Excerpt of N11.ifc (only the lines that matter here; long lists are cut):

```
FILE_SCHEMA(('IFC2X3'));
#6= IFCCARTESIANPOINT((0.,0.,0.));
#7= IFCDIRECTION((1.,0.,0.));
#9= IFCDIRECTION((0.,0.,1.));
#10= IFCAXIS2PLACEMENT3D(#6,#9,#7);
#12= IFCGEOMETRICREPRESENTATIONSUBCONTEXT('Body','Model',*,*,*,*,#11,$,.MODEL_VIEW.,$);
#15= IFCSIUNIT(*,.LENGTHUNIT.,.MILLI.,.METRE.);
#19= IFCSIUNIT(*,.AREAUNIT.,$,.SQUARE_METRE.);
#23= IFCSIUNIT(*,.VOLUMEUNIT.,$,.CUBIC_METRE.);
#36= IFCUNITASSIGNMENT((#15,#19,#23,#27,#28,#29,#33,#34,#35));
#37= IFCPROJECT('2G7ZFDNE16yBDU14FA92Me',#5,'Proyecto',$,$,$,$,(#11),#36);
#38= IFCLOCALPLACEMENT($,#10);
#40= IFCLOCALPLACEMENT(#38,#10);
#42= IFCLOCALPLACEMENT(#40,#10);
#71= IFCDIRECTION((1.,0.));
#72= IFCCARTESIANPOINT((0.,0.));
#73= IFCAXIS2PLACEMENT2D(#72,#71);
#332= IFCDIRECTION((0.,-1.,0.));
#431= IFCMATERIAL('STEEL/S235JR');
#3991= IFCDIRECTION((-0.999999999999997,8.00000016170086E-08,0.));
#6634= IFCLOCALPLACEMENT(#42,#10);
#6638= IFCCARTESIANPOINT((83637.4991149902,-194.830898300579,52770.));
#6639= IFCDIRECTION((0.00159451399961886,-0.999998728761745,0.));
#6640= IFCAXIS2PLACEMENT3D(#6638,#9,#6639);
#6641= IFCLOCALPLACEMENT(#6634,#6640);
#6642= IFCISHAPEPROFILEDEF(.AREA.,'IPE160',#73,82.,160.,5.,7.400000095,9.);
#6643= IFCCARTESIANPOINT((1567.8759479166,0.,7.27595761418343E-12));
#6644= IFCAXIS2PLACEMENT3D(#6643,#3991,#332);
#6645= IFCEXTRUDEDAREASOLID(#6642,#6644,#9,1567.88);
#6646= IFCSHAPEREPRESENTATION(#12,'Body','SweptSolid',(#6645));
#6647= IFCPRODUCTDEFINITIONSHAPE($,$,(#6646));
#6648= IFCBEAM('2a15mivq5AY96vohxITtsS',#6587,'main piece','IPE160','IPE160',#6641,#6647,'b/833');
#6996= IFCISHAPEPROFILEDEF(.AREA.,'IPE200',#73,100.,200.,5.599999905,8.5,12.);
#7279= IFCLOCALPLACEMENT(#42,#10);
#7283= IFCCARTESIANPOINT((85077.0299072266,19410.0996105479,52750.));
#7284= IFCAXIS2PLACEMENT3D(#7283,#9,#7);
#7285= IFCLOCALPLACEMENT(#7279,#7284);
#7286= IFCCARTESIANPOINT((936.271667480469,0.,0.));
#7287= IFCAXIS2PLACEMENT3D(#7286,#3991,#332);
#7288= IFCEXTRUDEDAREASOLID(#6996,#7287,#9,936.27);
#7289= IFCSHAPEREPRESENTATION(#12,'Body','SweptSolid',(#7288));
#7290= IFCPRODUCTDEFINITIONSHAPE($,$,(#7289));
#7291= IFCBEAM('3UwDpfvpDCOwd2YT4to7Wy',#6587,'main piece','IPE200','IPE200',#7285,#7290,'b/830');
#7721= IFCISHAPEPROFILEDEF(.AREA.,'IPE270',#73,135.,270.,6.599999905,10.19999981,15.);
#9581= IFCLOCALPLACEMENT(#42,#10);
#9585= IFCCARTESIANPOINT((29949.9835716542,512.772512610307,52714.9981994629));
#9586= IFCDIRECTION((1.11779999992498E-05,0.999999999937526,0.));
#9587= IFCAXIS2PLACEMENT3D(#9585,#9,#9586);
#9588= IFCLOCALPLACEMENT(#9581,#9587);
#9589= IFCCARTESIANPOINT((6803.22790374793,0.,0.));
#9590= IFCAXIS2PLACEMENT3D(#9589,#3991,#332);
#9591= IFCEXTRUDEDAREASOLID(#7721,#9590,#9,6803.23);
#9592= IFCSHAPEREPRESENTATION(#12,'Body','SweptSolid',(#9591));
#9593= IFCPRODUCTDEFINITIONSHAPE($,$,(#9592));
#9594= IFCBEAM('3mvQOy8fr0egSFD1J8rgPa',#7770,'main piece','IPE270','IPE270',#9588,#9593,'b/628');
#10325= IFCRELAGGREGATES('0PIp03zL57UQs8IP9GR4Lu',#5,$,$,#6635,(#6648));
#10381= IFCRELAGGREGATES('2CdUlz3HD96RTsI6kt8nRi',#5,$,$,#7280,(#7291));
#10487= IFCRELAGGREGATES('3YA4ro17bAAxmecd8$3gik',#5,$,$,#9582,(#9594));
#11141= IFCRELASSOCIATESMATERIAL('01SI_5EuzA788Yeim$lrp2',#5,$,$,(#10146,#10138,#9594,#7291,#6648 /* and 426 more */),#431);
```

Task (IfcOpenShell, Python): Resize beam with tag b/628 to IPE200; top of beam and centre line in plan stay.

```python
import ifcopenshell
import ifcopenshell.util.element
import ifcopenshell.util.representation

model = ifcopenshell.open("N11.ifc")

member = model.by_guid("3mvQOy8fr0egSFD1J8rgPa")
source = next(p for p in model.by_type("IfcIShapeProfileDef") if p.ProfileName == "IPE200")

body = ifcopenshell.util.representation.get_representation(member, "Model", "Body")
solid = body.Items[0]
old_profile = solid.SweptArea

# Copy the section's sizes but keep this member's own profile position.
profile = ifcopenshell.util.element.copy(model, source)
# Profiles are centred, so shift by half the change in depth to hold the top.
shift = (old_profile.OverallDepth - profile.OverallDepth) / 2
x, y = old_profile.Position.Location.Coordinates
up = (0.0, 1.0)  # upwards, in the solid's own plane
location = model.createIfcCartesianPoint((x + up[0] * shift, y + up[1] * shift))
profile.Position = model.createIfcAxis2Placement2D(location, old_profile.Position.RefDirection)
solid.SweptArea = profile
if not model.get_total_inverses(old_profile):
    ifcopenshell.util.element.remove_deep2(model, old_profile)
member.Description = member.Description.replace("IPE270", "IPE200")
member.ObjectType = member.ObjectType.replace("IPE270", "IPE200")

print(solid.SweptArea)

model.write("N11-out.ifc")
```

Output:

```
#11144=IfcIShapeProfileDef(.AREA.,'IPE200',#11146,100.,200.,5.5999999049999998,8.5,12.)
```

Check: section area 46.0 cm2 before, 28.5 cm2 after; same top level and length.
